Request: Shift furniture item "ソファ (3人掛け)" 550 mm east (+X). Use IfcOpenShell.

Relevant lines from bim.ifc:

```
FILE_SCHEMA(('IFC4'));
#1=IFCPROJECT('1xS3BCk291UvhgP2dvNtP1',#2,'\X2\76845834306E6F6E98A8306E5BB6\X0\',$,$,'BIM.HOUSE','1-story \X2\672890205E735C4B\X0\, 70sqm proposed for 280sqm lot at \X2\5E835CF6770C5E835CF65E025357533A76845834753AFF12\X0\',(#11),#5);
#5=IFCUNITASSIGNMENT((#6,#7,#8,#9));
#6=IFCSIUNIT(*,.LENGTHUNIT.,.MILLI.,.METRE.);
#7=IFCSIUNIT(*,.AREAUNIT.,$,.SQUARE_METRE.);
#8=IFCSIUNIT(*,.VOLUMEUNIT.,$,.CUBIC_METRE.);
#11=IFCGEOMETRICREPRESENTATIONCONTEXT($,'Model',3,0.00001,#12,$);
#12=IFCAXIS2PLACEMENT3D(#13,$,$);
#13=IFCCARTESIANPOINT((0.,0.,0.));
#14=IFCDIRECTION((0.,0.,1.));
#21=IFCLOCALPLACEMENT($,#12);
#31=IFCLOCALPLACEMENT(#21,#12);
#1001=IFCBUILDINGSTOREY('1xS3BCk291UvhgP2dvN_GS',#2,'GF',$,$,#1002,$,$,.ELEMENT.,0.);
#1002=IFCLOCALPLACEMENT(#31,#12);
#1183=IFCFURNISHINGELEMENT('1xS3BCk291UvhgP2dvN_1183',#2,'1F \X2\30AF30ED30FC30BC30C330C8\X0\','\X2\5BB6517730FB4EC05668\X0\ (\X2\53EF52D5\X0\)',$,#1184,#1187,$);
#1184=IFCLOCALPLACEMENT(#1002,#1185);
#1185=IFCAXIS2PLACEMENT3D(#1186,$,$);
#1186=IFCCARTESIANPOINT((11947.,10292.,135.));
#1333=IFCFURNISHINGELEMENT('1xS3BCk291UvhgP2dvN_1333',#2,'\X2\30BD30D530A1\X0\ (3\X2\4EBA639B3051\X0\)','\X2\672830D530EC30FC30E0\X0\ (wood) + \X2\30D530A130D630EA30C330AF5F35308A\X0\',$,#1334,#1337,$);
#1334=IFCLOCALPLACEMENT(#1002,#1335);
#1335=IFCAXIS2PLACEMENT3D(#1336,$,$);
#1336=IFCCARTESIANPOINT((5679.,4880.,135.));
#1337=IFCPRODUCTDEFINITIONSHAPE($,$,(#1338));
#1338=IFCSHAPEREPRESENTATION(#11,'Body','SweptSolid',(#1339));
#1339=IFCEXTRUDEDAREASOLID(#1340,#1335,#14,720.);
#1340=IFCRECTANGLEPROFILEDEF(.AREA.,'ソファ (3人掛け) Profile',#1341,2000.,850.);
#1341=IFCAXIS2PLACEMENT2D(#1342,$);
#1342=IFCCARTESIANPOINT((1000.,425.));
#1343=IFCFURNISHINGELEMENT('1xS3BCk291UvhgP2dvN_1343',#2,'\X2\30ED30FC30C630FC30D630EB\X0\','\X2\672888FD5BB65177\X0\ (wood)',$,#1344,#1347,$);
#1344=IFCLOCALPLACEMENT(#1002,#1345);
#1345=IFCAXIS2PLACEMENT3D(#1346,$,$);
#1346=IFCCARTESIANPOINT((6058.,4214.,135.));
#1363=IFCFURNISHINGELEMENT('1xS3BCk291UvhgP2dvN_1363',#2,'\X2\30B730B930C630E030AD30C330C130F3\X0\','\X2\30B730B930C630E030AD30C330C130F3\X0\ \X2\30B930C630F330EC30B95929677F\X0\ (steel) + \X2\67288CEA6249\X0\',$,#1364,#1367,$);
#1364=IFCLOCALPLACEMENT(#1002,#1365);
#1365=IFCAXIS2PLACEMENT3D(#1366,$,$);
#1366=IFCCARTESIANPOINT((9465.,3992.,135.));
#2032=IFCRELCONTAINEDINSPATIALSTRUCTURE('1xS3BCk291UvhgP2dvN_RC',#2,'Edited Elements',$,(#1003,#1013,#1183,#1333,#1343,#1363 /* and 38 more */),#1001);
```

```python
import ifcopenshell
import ifcopenshell.api.geometry
import ifcopenshell.util.placement
import ifcopenshell.util.unit

model = ifcopenshell.open("bim.ifc")
unit_scale = ifcopenshell.util.unit.calculate_unit_scale(model)

item = model.by_id(1333)
matrix = ifcopenshell.util.placement.get_local_placement(item.ObjectPlacement)
matrix[0, 3] += 0.55 / unit_scale
ifcopenshell.api.geometry.edit_object_placement(model, product=item, matrix=matrix, is_si=False)

print(ifcopenshell.util.placement.get_local_placement(item.ObjectPlacement).round(3) + 0.0)

model.write("bim_v2.ifc")
```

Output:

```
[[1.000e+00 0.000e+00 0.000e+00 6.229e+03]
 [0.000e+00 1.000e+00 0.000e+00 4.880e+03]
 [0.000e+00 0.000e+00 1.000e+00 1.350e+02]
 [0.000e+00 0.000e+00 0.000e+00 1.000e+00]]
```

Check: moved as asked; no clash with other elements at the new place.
